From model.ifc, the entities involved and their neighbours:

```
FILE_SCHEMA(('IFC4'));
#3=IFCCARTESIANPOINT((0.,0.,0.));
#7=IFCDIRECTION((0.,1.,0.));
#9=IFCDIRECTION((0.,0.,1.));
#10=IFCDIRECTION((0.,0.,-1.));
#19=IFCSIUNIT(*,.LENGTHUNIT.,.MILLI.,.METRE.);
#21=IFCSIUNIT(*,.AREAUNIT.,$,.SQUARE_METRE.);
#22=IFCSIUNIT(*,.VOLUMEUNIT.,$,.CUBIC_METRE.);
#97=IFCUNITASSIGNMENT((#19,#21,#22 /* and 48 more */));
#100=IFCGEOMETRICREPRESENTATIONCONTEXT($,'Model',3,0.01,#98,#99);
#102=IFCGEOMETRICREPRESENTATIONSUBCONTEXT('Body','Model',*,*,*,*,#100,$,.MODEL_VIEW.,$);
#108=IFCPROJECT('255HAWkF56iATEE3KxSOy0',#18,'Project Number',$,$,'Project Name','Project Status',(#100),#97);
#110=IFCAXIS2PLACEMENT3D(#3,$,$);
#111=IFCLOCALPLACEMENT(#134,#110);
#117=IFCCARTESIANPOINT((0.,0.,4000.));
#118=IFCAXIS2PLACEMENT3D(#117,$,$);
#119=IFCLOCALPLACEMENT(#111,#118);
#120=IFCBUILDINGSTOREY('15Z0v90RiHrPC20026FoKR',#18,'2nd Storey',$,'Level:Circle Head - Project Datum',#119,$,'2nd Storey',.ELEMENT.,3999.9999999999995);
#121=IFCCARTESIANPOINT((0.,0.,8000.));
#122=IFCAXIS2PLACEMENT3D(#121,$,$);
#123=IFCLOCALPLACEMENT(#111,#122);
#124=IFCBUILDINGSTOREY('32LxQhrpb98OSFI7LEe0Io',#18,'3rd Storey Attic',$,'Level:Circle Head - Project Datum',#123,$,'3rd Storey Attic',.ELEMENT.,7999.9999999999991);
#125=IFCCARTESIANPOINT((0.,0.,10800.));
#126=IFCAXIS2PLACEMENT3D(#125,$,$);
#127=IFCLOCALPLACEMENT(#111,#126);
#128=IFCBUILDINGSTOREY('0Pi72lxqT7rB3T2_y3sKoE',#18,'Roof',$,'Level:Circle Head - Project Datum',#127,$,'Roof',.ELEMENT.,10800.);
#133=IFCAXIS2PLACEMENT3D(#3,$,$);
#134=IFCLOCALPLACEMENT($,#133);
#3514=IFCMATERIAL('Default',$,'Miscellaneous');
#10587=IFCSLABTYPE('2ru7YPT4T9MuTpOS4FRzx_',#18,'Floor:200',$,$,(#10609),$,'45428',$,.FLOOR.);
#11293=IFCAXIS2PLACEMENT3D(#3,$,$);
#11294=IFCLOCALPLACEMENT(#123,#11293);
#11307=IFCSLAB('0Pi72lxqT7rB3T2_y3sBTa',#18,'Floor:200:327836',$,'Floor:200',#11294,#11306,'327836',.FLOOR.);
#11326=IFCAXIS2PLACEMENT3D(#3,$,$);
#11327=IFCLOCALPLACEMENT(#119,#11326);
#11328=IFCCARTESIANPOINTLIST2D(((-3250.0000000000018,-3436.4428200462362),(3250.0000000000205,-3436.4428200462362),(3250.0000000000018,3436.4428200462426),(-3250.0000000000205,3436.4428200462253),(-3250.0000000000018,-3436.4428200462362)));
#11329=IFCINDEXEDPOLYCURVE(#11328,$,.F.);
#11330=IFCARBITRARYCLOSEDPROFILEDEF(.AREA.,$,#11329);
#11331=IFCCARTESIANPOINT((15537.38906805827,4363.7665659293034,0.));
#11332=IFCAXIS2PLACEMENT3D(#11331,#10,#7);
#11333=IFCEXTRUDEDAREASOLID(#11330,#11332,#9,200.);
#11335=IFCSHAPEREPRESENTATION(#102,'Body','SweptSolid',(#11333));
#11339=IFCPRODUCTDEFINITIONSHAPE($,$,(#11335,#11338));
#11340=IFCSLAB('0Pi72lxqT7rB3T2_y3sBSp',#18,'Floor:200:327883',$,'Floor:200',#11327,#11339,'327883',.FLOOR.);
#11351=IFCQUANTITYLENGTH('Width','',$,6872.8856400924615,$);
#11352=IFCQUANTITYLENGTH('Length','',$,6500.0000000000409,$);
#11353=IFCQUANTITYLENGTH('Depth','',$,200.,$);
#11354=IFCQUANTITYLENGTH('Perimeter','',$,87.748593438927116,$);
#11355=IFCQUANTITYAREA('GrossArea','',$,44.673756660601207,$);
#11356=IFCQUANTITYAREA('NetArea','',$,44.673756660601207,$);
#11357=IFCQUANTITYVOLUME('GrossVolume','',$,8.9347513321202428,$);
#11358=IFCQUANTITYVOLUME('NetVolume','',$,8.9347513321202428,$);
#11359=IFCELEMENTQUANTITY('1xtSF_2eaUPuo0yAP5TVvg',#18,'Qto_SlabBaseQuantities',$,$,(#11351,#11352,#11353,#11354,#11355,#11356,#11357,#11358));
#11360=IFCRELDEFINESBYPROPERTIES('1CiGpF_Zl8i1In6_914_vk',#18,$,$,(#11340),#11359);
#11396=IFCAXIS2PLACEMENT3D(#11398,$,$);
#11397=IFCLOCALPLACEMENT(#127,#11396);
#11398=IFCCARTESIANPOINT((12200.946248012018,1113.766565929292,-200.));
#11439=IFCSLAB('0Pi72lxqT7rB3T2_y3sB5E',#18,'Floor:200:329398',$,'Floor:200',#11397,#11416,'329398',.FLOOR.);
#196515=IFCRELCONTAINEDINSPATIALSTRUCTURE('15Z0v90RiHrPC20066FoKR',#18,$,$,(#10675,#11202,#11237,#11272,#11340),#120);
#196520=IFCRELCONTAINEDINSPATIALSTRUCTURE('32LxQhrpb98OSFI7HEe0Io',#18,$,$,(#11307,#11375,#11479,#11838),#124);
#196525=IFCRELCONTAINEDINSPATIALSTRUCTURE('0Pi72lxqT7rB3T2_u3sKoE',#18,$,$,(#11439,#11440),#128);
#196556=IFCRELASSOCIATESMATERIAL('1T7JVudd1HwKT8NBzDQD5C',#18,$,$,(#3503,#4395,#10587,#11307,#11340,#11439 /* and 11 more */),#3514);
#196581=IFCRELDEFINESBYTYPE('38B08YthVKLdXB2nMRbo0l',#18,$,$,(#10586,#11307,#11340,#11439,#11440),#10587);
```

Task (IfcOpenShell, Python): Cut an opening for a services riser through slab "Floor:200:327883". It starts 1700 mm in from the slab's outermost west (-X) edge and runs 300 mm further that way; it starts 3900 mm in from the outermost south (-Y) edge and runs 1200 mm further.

```python
import numpy as np
import ifcopenshell
import ifcopenshell.api.feature
import ifcopenshell.api.geometry
import ifcopenshell.api.pset
import ifcopenshell.api.root
import ifcopenshell.geom
import ifcopenshell.util.element
import ifcopenshell.util.placement
import ifcopenshell.util.representation
import ifcopenshell.util.shape
import ifcopenshell.util.unit

model = ifcopenshell.open("model.ifc")
unit_scale = ifcopenshell.util.unit.calculate_unit_scale(model)
area_scale = ifcopenshell.util.unit.calculate_unit_scale(model, "AREAUNIT")
volume_scale = ifcopenshell.util.unit.calculate_unit_scale(model, "VOLUMEUNIT")
settings = ifcopenshell.geom.settings()


def volume(element):
    """Net volume in cubic metres, openings subtracted."""
    shape = ifcopenshell.geom.create_shape(settings, element)
    return ifcopenshell.util.shape.get_volume(shape.geometry)


slab = model.by_guid("0Pi72lxqT7rB3T2_y3sBSp")
before = volume(slab)

# Extent in the slab's own axes, in metres. The edges named are its -X and -Y sides.
slab_shape = ifcopenshell.geom.create_shape(settings, slab)
vertices = ifcopenshell.util.shape.get_vertices(slab_shape.geometry)
x_min, y_min, bottom = vertices.min(axis=0)
top = vertices[:, 2].max()

opening = ifcopenshell.api.root.create_entity(model, ifc_class="IfcOpeningElement", name="Services riser opening", predefined_type="OPENING")
context = ifcopenshell.util.representation.get_context(model, "Model", "Body", "MODEL_VIEW")
width, depth = 0.3, 1.2
outline = [(0.0, 0.0), (width, 0.0), (width, depth), (0.0, depth), (0.0, 0.0)]
# Overshoot both faces by 50 mm so the cut is clean.
shape = ifcopenshell.api.geometry.add_slab_representation(
    model, context=context, depth=top - bottom + 0.1, polyline=outline
)
ifcopenshell.api.geometry.assign_representation(model, product=opening, representation=shape)

matrix = ifcopenshell.util.placement.get_local_placement(slab.ObjectPlacement)
matrix[:, 3] = matrix @ np.append(np.array([x_min + 1.7, y_min + 3.9, bottom - 0.05]) / unit_scale, 1.0)
ifcopenshell.api.geometry.edit_object_placement(model, product=opening, matrix=matrix, is_si=False)
ifcopenshell.api.feature.add_feature(model, feature=opening, element=slab)

after = volume(slab)

# Update the slab's stored quantities.
qto = model.by_id(ifcopenshell.util.element.get_pset(slab, "Qto_SlabBaseQuantities", should_inherit=False)["id"])
ifcopenshell.api.pset.edit_qto(model, qto=qto, properties={
    "NetArea": after / (top - bottom) / area_scale,
    "NetVolume": after / volume_scale,
})

print(f"slab volume {before:.3f} -> {after:.3f} m3")

model.write("model-out.ifc")
```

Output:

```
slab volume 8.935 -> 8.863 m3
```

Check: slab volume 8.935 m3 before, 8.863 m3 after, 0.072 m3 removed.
